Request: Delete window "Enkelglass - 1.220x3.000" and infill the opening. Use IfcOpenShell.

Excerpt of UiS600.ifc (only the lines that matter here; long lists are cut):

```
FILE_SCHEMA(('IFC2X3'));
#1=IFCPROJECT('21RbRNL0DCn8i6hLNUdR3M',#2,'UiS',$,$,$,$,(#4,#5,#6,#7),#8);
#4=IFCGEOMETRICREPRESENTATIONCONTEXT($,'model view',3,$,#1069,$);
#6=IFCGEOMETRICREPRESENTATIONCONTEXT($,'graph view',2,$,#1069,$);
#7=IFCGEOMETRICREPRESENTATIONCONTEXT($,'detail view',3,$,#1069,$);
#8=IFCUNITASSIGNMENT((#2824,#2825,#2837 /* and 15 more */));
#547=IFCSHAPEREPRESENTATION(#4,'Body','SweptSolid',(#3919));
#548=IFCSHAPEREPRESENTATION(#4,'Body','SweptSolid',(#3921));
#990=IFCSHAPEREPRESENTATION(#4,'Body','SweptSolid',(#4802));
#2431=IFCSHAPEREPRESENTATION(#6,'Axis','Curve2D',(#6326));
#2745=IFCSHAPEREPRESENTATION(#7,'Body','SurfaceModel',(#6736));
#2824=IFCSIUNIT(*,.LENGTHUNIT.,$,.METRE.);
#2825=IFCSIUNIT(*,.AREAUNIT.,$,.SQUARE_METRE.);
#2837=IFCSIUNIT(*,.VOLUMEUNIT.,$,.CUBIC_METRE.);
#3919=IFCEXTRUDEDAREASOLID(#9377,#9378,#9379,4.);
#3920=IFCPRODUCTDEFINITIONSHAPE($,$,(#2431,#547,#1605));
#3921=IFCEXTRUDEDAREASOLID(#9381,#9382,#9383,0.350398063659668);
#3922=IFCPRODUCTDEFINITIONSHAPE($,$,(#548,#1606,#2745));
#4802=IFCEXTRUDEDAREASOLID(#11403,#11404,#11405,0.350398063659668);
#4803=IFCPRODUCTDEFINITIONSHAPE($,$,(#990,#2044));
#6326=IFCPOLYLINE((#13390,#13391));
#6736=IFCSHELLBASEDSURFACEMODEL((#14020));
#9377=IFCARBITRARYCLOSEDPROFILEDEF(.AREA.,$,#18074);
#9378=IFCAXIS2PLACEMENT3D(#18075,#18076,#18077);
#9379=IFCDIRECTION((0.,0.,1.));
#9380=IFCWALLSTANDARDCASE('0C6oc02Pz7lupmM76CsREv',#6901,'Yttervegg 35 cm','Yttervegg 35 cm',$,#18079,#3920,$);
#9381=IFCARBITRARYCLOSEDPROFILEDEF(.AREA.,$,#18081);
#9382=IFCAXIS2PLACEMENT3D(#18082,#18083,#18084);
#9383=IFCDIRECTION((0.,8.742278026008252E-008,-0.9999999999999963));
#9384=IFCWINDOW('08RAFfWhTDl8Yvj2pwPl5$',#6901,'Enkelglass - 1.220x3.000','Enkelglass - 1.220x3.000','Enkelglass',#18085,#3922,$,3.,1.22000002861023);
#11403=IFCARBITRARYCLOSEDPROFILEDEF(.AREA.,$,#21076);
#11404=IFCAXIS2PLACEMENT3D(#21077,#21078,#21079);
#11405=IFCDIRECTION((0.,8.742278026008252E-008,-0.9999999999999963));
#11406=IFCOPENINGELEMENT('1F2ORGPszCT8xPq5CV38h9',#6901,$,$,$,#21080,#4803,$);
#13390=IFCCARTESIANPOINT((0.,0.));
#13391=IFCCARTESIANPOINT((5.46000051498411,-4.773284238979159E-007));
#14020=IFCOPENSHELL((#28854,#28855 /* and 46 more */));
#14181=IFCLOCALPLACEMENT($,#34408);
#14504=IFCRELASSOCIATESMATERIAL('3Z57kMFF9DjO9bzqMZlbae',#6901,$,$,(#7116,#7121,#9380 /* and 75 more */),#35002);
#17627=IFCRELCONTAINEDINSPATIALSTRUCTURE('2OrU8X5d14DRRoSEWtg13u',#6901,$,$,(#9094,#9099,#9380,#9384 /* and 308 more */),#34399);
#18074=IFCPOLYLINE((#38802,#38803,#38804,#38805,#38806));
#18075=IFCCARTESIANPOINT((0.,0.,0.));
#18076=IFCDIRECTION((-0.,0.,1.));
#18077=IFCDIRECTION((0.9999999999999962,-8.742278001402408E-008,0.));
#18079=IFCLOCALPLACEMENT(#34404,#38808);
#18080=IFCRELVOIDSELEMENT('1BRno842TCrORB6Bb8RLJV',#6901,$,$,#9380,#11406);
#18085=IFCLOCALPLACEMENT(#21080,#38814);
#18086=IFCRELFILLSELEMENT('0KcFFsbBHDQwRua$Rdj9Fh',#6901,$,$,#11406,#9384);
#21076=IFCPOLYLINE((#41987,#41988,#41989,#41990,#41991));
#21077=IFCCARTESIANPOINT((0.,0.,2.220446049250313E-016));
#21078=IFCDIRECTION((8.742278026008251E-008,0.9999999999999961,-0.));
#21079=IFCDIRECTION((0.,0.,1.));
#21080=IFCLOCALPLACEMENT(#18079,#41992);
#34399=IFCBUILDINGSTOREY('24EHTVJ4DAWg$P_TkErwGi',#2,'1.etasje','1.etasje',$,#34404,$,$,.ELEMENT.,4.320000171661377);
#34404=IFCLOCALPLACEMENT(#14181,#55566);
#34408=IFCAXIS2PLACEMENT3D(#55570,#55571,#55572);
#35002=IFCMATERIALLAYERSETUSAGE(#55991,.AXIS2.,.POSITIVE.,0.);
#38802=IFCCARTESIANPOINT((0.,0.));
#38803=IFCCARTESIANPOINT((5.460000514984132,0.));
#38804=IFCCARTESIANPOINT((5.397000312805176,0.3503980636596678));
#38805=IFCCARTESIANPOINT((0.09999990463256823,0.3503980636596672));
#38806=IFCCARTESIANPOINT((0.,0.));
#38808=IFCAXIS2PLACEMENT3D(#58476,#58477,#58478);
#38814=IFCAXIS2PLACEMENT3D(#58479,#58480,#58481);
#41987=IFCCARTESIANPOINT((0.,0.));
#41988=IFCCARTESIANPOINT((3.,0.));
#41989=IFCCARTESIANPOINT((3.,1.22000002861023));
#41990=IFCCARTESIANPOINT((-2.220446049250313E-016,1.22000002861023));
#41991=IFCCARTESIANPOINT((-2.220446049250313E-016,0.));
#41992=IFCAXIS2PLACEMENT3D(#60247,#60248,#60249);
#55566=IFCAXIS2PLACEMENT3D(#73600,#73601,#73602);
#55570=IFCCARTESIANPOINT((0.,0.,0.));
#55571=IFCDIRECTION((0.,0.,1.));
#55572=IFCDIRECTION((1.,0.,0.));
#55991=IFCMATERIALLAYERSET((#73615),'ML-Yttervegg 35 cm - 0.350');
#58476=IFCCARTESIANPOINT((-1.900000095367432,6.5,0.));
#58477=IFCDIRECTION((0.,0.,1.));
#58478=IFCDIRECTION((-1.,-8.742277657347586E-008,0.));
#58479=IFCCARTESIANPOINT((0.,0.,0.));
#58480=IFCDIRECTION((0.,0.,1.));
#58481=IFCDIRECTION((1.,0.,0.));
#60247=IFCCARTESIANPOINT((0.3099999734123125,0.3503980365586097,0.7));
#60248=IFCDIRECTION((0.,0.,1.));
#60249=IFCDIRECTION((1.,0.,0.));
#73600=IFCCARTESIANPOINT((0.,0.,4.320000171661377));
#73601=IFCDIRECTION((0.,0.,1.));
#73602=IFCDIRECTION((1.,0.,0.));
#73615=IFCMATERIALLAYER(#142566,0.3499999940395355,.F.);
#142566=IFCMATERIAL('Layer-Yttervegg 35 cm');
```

```python
import ifcopenshell
import ifcopenshell.api.feature
import ifcopenshell.api.root
import ifcopenshell.geom
import ifcopenshell.util.shape

model = ifcopenshell.open("UiS600.ifc")
settings = ifcopenshell.geom.settings()


def volume(element):
    """Net volume in cubic metres, openings subtracted."""
    shape = ifcopenshell.geom.create_shape(settings, element)
    return ifcopenshell.util.shape.get_volume(shape.geometry)


window = model.by_guid("08RAFfWhTDl8Yvj2pwPl5$")
opening = window.FillsVoids[0].RelatingOpeningElement
wall = opening.VoidsElements[0].RelatingBuildingElement
before = volume(wall)

ifcopenshell.api.root.remove_product(model, product=window)
ifcopenshell.api.feature.remove_feature(model, feature=opening)

after = volume(wall)

print(f"wall volume {before:.3f} -> {after:.3f} m3")

model.write("UiS600_edited.ifc")
```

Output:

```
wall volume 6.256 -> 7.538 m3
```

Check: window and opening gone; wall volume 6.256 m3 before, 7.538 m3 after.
